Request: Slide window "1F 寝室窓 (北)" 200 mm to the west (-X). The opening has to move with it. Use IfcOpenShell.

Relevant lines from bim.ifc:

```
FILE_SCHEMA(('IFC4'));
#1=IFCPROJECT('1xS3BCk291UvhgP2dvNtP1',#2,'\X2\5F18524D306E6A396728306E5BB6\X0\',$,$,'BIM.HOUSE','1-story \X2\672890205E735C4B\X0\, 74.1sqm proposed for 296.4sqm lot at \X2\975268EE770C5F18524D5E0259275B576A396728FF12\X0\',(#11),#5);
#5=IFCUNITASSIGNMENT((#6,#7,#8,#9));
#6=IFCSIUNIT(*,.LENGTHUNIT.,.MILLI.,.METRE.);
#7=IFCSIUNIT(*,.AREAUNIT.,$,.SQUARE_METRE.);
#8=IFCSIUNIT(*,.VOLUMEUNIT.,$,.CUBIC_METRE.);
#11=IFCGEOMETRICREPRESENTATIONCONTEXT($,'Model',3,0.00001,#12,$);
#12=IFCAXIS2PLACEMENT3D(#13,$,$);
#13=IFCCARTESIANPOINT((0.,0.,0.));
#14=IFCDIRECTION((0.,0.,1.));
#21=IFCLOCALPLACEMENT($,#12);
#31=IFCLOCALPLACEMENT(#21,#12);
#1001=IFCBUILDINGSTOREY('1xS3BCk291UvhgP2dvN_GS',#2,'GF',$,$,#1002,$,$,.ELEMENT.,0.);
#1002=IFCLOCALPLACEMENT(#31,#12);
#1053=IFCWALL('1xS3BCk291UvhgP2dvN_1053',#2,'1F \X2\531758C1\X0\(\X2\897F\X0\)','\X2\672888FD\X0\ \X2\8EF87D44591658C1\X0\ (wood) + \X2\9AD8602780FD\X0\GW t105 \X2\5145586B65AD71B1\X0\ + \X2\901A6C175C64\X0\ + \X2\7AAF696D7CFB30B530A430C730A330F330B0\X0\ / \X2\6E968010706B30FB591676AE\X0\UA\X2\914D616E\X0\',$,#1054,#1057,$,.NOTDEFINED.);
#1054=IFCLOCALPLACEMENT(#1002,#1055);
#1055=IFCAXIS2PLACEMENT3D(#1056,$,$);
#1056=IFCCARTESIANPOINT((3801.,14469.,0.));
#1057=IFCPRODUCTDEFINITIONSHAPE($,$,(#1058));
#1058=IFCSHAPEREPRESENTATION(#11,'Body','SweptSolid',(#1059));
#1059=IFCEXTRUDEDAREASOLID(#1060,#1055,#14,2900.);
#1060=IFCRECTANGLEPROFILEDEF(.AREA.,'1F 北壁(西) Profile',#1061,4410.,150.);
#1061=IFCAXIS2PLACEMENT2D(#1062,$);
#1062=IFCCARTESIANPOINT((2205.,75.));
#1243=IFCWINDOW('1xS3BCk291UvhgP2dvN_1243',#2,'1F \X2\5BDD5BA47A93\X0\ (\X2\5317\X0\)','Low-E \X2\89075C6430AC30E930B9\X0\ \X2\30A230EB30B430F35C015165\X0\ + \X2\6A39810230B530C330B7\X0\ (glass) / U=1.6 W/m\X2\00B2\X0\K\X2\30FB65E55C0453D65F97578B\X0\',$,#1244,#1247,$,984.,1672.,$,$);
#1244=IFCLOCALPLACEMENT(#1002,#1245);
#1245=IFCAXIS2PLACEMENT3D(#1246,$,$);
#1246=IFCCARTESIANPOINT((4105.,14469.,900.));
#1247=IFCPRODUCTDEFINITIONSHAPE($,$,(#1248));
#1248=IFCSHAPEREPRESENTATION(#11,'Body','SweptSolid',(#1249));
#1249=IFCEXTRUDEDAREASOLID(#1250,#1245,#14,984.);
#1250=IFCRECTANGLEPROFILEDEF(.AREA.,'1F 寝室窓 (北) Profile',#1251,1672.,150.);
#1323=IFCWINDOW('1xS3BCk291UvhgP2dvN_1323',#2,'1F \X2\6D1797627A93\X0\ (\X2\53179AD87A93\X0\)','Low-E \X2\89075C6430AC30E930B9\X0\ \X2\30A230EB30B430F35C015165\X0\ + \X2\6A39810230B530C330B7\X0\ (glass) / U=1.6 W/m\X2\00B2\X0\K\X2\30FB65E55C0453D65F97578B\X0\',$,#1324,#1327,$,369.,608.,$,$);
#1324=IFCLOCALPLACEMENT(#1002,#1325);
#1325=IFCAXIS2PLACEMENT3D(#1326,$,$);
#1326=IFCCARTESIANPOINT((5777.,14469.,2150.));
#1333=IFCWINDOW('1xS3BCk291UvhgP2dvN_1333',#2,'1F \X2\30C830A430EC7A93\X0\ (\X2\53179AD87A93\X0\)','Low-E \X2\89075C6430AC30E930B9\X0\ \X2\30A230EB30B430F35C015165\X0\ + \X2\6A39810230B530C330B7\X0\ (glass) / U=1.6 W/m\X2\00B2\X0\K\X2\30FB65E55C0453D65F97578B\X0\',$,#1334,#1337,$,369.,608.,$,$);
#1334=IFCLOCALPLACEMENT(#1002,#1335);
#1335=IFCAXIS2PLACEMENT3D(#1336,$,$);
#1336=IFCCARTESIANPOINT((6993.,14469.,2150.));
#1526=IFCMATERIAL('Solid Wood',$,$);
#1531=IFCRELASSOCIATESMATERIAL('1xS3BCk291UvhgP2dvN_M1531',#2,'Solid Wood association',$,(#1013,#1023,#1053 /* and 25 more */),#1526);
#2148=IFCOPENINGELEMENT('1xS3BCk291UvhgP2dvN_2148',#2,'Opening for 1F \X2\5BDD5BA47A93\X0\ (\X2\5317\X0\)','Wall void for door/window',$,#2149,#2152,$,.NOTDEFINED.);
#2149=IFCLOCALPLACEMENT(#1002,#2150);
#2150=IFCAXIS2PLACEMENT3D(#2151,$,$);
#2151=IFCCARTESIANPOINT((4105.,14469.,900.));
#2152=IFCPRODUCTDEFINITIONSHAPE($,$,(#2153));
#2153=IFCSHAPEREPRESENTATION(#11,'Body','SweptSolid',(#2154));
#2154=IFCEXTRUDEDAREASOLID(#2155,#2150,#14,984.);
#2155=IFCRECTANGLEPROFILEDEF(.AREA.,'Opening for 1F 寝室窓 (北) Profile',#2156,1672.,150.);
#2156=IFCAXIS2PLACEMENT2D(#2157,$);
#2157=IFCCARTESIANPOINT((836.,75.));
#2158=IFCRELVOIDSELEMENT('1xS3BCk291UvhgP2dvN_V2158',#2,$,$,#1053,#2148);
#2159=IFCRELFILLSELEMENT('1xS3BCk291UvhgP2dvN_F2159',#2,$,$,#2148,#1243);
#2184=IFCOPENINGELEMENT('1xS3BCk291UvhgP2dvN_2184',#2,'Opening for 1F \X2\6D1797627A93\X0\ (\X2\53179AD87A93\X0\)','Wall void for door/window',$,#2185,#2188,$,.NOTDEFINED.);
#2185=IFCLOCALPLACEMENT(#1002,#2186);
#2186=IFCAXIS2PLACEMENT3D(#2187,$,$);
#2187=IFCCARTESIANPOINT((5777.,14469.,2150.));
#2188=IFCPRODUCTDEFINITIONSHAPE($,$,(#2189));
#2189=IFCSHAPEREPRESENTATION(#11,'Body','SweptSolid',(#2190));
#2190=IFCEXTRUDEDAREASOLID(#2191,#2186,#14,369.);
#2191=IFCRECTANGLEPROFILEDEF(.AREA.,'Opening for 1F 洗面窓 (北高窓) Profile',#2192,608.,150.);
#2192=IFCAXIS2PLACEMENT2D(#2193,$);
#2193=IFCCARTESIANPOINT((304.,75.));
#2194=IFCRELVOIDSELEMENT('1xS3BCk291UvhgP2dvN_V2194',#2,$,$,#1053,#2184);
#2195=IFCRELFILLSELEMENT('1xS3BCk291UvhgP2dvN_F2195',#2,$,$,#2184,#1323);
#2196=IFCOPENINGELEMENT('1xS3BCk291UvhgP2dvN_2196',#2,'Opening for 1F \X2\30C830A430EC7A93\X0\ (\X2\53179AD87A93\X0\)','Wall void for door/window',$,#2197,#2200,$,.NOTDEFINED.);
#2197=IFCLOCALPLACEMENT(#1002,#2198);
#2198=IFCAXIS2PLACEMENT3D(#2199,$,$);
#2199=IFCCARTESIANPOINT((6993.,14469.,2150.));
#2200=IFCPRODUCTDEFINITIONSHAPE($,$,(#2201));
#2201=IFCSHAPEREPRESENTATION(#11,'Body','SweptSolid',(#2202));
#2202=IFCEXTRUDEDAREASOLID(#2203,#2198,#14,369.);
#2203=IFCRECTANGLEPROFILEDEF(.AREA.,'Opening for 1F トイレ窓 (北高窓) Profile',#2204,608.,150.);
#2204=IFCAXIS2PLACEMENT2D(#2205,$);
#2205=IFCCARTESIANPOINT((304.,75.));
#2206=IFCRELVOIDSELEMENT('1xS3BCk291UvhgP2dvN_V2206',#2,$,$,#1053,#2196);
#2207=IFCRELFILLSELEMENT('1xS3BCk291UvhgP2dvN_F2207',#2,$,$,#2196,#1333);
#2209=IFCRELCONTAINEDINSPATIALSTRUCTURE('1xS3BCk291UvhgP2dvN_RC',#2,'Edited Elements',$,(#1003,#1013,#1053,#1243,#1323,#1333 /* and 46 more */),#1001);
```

```python
import ifcopenshell
import ifcopenshell.api.geometry
import ifcopenshell.util.placement
import ifcopenshell.util.unit

model = ifcopenshell.open("bim.ifc")
unit_scale = ifcopenshell.util.unit.calculate_unit_scale(model)

window = model.by_guid("1xS3BCk291UvhgP2dvN_1243")
opening = window.FillsVoids[0].RelatingOpeningElement
wall = opening.VoidsElements[0].RelatingBuildingElement

wall_matrix = ifcopenshell.util.placement.get_local_placement(wall.ObjectPlacement)
shift = wall_matrix[:3, 0] * -0.2 / unit_scale
before = ifcopenshell.util.placement.get_local_placement(window.ObjectPlacement)[:3, 3].copy()

# The window is not placed relative to its opening, so move both.
for product in (opening, window):
    matrix = ifcopenshell.util.placement.get_local_placement(product.ObjectPlacement)
    matrix[:3, 3] += shift
    ifcopenshell.api.geometry.edit_object_placement(model, product=product, matrix=matrix, is_si=False)

after = ifcopenshell.util.placement.get_local_placement(window.ObjectPlacement)[:3, 3]
print("window moved by", (after - before).round(3) + 0.0)

model.write("bim_edited.ifc")
```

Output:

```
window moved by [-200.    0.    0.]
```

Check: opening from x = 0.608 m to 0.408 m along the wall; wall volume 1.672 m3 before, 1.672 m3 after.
